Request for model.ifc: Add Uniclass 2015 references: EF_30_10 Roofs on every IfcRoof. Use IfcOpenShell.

First a look at what the model holds.

```python
import ifcopenshell

model = ifcopenshell.open("model.ifc")
print(model.schema)
print("classifications:", [c.Name for c in model.by_type("IfcClassification")])
for ifc_class in ("IfcDoor", "IfcRoof", "IfcStair", "IfcWall", "IfcWindow"):
    print(ifc_class, len(model.by_type(ifc_class)))
```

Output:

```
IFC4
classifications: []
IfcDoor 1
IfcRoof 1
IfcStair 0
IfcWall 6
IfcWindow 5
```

```python
import ifcopenshell
import ifcopenshell.api.classification

model = ifcopenshell.open("model.ifc")

system = ifcopenshell.api.classification.add_classification(model, classification="Uniclass 2015")

codes = {
    "IfcRoof": ("EF_30_10", "Roofs"),
}
for ifc_class, (code, name) in codes.items():
    products = model.by_type(ifc_class)
    ifcopenshell.api.classification.add_reference(
        model, products=products, classification=system, identification=code, name=name
    )
    print(code, len(products))

model.write("model_v2.ifc")
```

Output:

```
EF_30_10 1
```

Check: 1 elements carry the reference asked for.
